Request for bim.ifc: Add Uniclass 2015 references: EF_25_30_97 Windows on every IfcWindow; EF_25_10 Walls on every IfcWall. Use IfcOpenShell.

First a look at what the model holds.

```python
import ifcopenshell

model = ifcopenshell.open("bim.ifc")
print(model.schema)
print("classifications:", [c.Name for c in model.by_type("IfcClassification")])
for ifc_class in ("IfcDoor", "IfcRoof", "IfcStair", "IfcWall", "IfcWindow"):
    print(ifc_class, len(model.by_type(ifc_class)))
```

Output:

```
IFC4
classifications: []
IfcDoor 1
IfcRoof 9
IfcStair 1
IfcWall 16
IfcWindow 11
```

```python
import ifcopenshell
import ifcopenshell.api.classification

model = ifcopenshell.open("bim.ifc")

system = ifcopenshell.api.classification.add_classification(model, classification="Uniclass 2015")

codes = {
    "IfcWindow": ("EF_25_30_97", "Windows"),
    "IfcWall": ("EF_25_10", "Walls"),
}
for ifc_class, (code, name) in codes.items():
    products = model.by_type(ifc_class)
    ifcopenshell.api.classification.add_reference(
        model, products=products, classification=system, identification=code, name=name
    )
    print(code, len(products))

model.write("bim_updated.ifc")
```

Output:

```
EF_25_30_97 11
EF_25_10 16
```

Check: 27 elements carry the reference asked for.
